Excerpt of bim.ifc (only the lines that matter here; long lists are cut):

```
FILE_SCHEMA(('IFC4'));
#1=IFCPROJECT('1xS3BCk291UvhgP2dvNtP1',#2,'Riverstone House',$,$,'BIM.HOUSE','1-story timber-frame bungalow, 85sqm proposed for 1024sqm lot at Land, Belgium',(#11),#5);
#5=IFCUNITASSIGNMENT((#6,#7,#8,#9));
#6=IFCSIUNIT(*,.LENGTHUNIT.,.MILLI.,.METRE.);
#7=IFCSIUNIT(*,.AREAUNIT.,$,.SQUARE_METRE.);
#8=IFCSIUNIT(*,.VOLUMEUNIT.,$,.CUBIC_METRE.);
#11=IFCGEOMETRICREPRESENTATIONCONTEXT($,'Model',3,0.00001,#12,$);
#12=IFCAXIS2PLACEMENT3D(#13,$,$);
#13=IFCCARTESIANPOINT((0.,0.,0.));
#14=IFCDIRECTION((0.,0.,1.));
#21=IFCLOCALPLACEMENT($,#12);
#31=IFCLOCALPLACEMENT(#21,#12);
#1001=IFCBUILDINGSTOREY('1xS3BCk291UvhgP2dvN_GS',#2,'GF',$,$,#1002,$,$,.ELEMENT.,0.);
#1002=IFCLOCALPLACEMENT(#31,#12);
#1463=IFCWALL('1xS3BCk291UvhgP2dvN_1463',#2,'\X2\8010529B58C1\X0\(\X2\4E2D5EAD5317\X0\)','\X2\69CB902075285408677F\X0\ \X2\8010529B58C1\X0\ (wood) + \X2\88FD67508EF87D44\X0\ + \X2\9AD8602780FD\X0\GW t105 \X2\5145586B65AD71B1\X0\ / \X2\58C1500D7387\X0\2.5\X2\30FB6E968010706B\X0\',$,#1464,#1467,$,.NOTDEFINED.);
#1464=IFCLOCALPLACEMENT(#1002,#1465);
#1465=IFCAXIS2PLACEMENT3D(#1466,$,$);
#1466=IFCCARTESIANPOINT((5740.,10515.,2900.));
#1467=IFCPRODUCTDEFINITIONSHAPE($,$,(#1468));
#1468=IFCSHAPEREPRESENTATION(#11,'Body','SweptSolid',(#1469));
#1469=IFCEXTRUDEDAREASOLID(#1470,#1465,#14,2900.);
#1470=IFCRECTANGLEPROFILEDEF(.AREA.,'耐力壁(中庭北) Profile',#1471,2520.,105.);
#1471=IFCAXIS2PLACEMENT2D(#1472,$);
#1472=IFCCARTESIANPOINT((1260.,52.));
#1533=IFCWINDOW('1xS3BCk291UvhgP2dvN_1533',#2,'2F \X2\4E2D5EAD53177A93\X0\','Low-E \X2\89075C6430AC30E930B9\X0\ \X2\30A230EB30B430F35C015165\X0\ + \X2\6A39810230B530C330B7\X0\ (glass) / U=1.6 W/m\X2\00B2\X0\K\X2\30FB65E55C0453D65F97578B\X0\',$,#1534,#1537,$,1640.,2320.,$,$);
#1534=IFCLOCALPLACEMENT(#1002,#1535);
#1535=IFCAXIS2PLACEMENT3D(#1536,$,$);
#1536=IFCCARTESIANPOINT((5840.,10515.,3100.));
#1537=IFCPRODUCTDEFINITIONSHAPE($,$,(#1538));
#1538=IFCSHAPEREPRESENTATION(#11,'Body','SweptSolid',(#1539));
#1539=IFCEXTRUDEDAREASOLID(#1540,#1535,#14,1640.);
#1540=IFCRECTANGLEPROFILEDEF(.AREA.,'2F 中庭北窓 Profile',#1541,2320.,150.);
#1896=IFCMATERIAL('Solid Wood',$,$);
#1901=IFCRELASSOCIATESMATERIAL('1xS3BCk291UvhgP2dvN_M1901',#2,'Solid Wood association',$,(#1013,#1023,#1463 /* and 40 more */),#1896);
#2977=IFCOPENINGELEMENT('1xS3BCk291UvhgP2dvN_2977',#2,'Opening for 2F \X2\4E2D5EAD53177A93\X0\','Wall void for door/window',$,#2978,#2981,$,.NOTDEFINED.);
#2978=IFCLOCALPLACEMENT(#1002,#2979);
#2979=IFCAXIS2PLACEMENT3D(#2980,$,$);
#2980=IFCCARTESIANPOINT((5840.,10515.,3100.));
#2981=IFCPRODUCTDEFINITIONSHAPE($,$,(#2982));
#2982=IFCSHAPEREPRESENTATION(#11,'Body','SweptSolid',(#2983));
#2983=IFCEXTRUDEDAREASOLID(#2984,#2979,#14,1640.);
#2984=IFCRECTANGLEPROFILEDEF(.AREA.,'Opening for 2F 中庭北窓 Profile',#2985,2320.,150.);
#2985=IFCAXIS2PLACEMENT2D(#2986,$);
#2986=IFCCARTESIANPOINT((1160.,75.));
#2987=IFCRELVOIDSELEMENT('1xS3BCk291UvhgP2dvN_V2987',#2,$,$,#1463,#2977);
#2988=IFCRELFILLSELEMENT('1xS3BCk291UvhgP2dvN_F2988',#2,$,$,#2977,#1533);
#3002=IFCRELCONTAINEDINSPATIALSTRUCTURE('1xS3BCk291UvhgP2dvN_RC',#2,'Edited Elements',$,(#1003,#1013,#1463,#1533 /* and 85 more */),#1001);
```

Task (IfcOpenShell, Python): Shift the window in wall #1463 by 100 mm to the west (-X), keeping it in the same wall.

```python
import ifcopenshell
import ifcopenshell.api.geometry
import ifcopenshell.util.placement
import ifcopenshell.util.unit

model = ifcopenshell.open("bim.ifc")
unit_scale = ifcopenshell.util.unit.calculate_unit_scale(model)

window = model.by_guid("1xS3BCk291UvhgP2dvN_1533")
opening = window.FillsVoids[0].RelatingOpeningElement
wall = opening.VoidsElements[0].RelatingBuildingElement

wall_matrix = ifcopenshell.util.placement.get_local_placement(wall.ObjectPlacement)
shift = wall_matrix[:3, 0] * -0.1 / unit_scale
before = ifcopenshell.util.placement.get_local_placement(window.ObjectPlacement)[:3, 3].copy()

# The window is not placed relative to its opening, so move both.
for product in (opening, window):
    matrix = ifcopenshell.util.placement.get_local_placement(product.ObjectPlacement)
    matrix[:3, 3] += shift
    ifcopenshell.api.geometry.edit_object_placement(model, product=product, matrix=matrix, is_si=False)

after = ifcopenshell.util.placement.get_local_placement(window.ObjectPlacement)[:3, 3]
print("window moved by", (after - before).round(3) + 0.0)

model.write("bim_updated.ifc")
```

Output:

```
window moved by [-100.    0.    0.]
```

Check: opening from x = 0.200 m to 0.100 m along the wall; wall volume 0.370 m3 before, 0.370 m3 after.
